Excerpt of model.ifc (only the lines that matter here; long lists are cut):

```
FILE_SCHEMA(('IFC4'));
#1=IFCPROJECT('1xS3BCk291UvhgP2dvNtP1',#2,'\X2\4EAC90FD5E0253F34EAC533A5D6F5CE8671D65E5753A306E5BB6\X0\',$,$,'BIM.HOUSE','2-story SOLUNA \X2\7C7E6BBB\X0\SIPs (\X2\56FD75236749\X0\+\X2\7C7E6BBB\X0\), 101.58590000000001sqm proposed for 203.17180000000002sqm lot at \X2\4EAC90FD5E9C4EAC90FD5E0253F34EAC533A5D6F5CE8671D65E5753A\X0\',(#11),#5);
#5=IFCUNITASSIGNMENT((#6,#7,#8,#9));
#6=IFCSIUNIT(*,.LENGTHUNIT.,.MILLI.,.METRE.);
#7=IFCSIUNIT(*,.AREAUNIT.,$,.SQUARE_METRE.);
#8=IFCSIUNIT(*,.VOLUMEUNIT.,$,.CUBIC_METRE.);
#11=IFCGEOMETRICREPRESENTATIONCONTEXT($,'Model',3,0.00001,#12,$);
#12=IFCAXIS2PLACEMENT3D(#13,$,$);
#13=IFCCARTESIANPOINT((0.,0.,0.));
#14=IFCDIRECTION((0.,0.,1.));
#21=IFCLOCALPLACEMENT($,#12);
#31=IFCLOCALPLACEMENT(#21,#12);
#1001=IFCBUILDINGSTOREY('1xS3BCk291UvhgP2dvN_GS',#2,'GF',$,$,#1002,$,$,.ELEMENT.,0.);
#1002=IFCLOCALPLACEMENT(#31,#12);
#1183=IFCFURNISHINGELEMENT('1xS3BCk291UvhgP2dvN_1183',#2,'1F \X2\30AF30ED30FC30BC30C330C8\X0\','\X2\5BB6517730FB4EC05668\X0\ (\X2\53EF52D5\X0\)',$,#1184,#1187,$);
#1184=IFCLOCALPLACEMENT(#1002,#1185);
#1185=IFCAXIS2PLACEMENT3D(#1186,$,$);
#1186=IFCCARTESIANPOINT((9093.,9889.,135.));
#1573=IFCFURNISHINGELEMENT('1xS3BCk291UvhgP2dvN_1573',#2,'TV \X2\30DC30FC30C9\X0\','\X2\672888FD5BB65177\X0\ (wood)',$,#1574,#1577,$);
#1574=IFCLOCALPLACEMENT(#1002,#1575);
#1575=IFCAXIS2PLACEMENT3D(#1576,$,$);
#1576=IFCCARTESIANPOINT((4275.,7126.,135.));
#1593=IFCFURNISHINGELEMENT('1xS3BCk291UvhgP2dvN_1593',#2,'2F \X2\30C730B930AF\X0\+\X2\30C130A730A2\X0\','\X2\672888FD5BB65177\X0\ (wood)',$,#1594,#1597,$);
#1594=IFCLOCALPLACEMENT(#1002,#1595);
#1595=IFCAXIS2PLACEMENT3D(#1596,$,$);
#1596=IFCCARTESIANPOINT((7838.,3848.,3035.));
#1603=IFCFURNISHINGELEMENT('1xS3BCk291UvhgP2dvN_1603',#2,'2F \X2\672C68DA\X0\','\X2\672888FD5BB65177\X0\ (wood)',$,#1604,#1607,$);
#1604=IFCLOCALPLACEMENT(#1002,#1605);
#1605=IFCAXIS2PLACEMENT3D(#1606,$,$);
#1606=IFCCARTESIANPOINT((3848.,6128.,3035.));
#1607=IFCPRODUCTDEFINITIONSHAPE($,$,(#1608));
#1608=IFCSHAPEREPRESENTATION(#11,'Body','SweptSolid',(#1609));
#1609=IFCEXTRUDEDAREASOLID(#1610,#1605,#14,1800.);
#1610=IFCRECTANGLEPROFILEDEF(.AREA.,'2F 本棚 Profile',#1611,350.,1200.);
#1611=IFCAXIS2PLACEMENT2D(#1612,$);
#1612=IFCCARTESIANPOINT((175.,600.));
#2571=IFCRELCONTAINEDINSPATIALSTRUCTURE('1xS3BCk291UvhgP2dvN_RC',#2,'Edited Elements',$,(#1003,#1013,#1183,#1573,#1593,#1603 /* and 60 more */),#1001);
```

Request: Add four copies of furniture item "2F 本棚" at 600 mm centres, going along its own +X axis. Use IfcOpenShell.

```python
import ifcopenshell
import ifcopenshell.api.geometry
import ifcopenshell.api.root
import ifcopenshell.util.element
import ifcopenshell.util.placement
import ifcopenshell.util.unit

model = ifcopenshell.open("model.ifc")
unit_scale = ifcopenshell.util.unit.calculate_unit_scale(model)


def reuse_history(source, copy):
    """copy_class also copies each property set's owner history, people and application; keep the originals."""
    for rel in copy.IsDefinedBy:
        if rel.is_a("IfcRelDefinesByProperties") and (history := rel.RelatingPropertyDefinition.OwnerHistory):
            rel.RelatingPropertyDefinition.OwnerHistory = source.OwnerHistory
            ifcopenshell.util.element.remove_deep2(model, history)


source = model.by_guid("1xS3BCk291UvhgP2dvN_1603")
base = ifcopenshell.util.placement.get_local_placement(source.ObjectPlacement)
step = base[:3, 0] * 0.6 / unit_scale

for i in range(1, 5):
    copy = ifcopenshell.api.root.copy_class(model, product=source)
    copy.Representation = ifcopenshell.util.element.copy_deep(
        model, source.Representation, exclude=["IfcGeometricRepresentationContext", "IfcRepresentationMap"]
    )
    reuse_history(source, copy)
    matrix = base.copy()
    matrix[:3, 3] += i * step
    print("added at", matrix[:3, 3].round(3) + 0.0)
    ifcopenshell.api.geometry.edit_object_placement(model, product=copy, matrix=matrix, is_si=False)

model.write("model_edited.ifc")
```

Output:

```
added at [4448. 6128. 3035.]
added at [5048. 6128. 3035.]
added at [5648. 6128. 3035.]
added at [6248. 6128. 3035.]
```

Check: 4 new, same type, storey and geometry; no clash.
